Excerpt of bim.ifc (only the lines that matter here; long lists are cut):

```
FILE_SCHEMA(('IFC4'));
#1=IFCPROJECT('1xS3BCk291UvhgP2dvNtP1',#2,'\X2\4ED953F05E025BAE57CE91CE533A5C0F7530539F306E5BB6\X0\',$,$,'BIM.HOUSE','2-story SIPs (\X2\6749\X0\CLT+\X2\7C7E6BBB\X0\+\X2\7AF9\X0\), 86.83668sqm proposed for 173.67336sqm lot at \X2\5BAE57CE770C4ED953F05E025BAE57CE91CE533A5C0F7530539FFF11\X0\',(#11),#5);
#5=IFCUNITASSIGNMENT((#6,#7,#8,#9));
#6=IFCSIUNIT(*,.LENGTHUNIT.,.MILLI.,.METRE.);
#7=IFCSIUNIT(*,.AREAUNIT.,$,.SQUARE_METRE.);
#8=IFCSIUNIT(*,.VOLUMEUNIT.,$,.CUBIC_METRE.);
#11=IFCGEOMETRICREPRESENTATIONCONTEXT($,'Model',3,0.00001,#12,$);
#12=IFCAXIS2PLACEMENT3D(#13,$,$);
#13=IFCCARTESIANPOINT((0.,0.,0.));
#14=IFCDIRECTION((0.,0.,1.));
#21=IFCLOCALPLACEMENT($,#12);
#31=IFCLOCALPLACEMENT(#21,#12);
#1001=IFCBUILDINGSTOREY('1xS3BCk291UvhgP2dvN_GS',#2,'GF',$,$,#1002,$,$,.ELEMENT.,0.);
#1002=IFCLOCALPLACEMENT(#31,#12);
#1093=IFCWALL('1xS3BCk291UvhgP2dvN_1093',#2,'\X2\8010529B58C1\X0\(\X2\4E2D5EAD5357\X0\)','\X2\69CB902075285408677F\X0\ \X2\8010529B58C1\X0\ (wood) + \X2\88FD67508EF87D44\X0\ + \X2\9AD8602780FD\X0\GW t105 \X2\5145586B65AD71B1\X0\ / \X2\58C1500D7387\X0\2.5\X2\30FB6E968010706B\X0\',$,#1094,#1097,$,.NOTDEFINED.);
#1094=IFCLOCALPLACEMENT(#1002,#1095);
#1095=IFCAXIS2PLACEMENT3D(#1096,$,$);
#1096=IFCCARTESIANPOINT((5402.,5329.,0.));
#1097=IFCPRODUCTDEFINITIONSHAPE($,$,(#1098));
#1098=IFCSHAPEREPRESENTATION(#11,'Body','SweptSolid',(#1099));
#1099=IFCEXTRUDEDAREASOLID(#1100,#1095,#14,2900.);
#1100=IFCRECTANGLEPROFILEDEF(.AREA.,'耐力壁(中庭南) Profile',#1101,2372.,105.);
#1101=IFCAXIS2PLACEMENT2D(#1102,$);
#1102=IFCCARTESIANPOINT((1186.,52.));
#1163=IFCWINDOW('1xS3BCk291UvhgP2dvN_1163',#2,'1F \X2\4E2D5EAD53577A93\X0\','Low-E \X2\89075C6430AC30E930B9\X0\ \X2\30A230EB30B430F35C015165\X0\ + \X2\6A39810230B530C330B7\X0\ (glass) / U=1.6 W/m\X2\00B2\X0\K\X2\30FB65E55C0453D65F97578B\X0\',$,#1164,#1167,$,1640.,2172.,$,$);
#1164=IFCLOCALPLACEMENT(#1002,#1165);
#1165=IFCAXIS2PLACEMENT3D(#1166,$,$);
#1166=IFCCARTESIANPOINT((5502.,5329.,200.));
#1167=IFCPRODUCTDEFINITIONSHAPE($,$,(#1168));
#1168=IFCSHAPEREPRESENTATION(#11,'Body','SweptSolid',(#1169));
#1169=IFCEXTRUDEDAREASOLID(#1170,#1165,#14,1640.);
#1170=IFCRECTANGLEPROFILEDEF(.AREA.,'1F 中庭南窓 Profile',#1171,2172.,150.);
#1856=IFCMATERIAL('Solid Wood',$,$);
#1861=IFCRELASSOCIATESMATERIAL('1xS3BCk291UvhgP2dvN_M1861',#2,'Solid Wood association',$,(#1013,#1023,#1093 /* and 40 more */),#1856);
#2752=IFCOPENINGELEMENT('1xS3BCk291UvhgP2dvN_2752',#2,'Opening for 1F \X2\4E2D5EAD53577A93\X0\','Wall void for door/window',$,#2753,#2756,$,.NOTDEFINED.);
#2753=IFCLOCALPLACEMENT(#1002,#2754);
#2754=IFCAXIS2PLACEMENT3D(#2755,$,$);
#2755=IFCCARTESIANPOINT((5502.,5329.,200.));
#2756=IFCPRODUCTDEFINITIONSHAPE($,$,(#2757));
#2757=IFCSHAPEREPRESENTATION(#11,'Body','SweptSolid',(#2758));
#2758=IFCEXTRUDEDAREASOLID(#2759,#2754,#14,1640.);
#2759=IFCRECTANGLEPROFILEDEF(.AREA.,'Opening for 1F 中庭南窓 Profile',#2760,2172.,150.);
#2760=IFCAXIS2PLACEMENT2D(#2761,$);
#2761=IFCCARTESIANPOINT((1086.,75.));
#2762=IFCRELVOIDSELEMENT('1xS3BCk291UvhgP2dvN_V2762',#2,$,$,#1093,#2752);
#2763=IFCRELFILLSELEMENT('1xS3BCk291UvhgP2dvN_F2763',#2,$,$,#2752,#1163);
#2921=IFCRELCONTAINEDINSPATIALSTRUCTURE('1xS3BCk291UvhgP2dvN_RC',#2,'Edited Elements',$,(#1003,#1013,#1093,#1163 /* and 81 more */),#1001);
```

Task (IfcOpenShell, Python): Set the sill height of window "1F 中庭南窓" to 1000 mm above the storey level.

```python
import numpy as np
import ifcopenshell
import ifcopenshell.api.geometry
import ifcopenshell.geom
import ifcopenshell.util.element
import ifcopenshell.util.placement
import ifcopenshell.util.shape
import ifcopenshell.util.unit

model = ifcopenshell.open("bim.ifc")
unit_scale = ifcopenshell.util.unit.calculate_unit_scale(model)

window = model.by_id(1163)
opening = window.FillsVoids[0].RelatingOpeningElement
storey = ifcopenshell.util.element.get_container(window, ifc_class="IfcBuildingStorey")
level = ifcopenshell.util.placement.get_local_placement(storey.ObjectPlacement)[2, 3]

# The opening's origin need not be at the sill, so measure its lowest point.
shape = ifcopenshell.geom.create_shape(ifcopenshell.geom.settings(), opening)
bottom = ifcopenshell.util.shape.get_shape_bottom_elevation(shape, shape.geometry) / unit_scale
dz = level + 1000.0 - bottom

shift = np.array([0.0, 0.0, dz])
# The window is not placed relative to its opening, so move both.
for product in (opening, window):
    matrix = ifcopenshell.util.placement.get_local_placement(product.ObjectPlacement)
    matrix[:3, 3] += shift
    ifcopenshell.api.geometry.edit_object_placement(model, product=product, matrix=matrix, is_si=False)

print(f"moved by {dz * unit_scale:+.3f} m")

model.write("bim-out.ifc")
```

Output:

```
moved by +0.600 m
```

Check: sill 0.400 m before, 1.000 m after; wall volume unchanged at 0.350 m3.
